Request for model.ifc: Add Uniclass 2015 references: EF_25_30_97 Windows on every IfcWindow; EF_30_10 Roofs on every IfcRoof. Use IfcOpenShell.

First a look at what the model holds.

```python
import ifcopenshell

model = ifcopenshell.open("model.ifc")
print(model.schema)
print("classifications:", [c.Name for c in model.by_type("IfcClassification")])
for ifc_class in ("IfcDoor", "IfcRoof", "IfcStair", "IfcWall", "IfcWindow"):
    print(ifc_class, len(model.by_type(ifc_class)))
```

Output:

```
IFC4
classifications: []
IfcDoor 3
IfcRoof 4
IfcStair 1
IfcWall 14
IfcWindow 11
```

```python
import ifcopenshell
import ifcopenshell.api.classification

model = ifcopenshell.open("model.ifc")

system = ifcopenshell.api.classification.add_classification(model, classification="Uniclass 2015")

codes = {
    "IfcWindow": ("EF_25_30_97", "Windows"),
    "IfcRoof": ("EF_30_10", "Roofs"),
}
for ifc_class, (code, name) in codes.items():
    products = model.by_type(ifc_class)
    ifcopenshell.api.classification.add_reference(
        model, products=products, classification=system, identification=code, name=name
    )
    print(code, len(products))

model.write("model_edited.ifc")
```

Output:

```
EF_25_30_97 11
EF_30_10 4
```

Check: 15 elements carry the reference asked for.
